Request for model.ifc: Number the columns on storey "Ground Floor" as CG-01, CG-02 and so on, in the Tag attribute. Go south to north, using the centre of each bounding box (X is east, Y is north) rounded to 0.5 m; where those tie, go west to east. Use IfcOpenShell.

First a look at what the model holds.

```python
import ifcopenshell
import ifcopenshell.util.element
import ifcopenshell.util.placement

model = ifcopenshell.open("model.ifc")
print(model.schema)
storey = next(s for s in model.by_type("IfcBuildingStorey") if s.Name == "Ground Floor")
columns = [e for e in ifcopenshell.util.element.get_decomposition(storey) if e.is_a("IfcColumn")]
for e in sorted(columns, key=lambda e: e.id()):
    origin = ifcopenshell.util.placement.get_local_placement(e.ObjectPlacement)[:3, 3]
    print(e.id(), e.Tag, e.Name, origin.round(2) + 0.0, sep=" | ")
```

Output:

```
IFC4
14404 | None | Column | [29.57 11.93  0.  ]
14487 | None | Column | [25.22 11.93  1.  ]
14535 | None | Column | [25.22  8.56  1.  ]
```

```python
import ifcopenshell
import ifcopenshell.geom
import ifcopenshell.util.element
import ifcopenshell.util.shape

model = ifcopenshell.open("model.ifc")
settings = ifcopenshell.geom.settings()
settings.set("use-world-coords", True)


def centre(element):
    shape = ifcopenshell.geom.create_shape(settings, element)
    return ifcopenshell.util.shape.get_bbox_centroid(shape.geometry)


storey = next(s for s in model.by_type("IfcBuildingStorey") if s.Name == "Ground Floor")
columns = [e for e in ifcopenshell.util.element.get_decomposition(storey) if e.is_a("IfcColumn")]

# Insertion points can sit at a corner or the storey origin, so sort by the geometry (in metres).
centres = {e: centre(e) for e in columns}
columns.sort(key=lambda e: (round(centres[e][1] / 0.5), centres[e][0]))

for i, e in enumerate(columns, start=1):
    number = f"CG-{i:02d}"
    e.Tag = number
    print(e.id(), number)

model.write("model_rev.ifc")
```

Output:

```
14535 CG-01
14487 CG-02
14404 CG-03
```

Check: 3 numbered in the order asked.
